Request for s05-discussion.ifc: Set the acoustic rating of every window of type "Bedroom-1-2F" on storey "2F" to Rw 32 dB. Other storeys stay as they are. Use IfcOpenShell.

First a look at what the model holds.

```python
import ifcopenshell
import ifcopenshell.util.element

model = ifcopenshell.open("s05-discussion.ifc")
print(model.schema)
storey = next(s for s in model.by_type("IfcBuildingStorey") if s.Name == "2F")
windows = [e for e in ifcopenshell.util.element.get_decomposition(storey) if e.is_a("IfcWindow")]
seen = {}
for e in windows:
    element_type = ifcopenshell.util.element.get_type(e)
    key = (element_type.Name if element_type != e and element_type else None, ifcopenshell.util.element.get_pset(e, "Pset_WindowCommon", "AcousticRating"))
    seen[key] = seen.get(key, 0) + 1
for (name, value), count in sorted(seen.items(), key=str):
    print(count, "x", name, "|", value)
```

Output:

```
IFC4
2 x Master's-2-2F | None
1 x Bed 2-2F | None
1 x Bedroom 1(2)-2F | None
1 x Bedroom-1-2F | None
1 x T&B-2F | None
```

```python
import ifcopenshell
import ifcopenshell.api.pset
import ifcopenshell.util.element

model = ifcopenshell.open("s05-discussion.ifc")

storey = next(s for s in model.by_type("IfcBuildingStorey") if s.Name == "2F")
windows = [e for e in ifcopenshell.util.element.get_decomposition(storey) if e.is_a("IfcWindow")]

count = 0
for e in windows:
    element_type = ifcopenshell.util.element.get_type(e)
    if element_type in (None, e) or element_type.Name != "Bedroom-1-2F":
        continue
    # add_pset returns the element's existing set when there is one.
    pset = ifcopenshell.api.pset.add_pset(model, product=e, name="Pset_WindowCommon")
    ifcopenshell.api.pset.edit_pset(model, pset=pset, properties={"AcousticRating": "Rw 32 dB"})
    count += 1

print(count, "windows updated")

model.write("s05-discussion_edited.ifc")
```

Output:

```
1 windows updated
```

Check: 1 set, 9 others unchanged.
